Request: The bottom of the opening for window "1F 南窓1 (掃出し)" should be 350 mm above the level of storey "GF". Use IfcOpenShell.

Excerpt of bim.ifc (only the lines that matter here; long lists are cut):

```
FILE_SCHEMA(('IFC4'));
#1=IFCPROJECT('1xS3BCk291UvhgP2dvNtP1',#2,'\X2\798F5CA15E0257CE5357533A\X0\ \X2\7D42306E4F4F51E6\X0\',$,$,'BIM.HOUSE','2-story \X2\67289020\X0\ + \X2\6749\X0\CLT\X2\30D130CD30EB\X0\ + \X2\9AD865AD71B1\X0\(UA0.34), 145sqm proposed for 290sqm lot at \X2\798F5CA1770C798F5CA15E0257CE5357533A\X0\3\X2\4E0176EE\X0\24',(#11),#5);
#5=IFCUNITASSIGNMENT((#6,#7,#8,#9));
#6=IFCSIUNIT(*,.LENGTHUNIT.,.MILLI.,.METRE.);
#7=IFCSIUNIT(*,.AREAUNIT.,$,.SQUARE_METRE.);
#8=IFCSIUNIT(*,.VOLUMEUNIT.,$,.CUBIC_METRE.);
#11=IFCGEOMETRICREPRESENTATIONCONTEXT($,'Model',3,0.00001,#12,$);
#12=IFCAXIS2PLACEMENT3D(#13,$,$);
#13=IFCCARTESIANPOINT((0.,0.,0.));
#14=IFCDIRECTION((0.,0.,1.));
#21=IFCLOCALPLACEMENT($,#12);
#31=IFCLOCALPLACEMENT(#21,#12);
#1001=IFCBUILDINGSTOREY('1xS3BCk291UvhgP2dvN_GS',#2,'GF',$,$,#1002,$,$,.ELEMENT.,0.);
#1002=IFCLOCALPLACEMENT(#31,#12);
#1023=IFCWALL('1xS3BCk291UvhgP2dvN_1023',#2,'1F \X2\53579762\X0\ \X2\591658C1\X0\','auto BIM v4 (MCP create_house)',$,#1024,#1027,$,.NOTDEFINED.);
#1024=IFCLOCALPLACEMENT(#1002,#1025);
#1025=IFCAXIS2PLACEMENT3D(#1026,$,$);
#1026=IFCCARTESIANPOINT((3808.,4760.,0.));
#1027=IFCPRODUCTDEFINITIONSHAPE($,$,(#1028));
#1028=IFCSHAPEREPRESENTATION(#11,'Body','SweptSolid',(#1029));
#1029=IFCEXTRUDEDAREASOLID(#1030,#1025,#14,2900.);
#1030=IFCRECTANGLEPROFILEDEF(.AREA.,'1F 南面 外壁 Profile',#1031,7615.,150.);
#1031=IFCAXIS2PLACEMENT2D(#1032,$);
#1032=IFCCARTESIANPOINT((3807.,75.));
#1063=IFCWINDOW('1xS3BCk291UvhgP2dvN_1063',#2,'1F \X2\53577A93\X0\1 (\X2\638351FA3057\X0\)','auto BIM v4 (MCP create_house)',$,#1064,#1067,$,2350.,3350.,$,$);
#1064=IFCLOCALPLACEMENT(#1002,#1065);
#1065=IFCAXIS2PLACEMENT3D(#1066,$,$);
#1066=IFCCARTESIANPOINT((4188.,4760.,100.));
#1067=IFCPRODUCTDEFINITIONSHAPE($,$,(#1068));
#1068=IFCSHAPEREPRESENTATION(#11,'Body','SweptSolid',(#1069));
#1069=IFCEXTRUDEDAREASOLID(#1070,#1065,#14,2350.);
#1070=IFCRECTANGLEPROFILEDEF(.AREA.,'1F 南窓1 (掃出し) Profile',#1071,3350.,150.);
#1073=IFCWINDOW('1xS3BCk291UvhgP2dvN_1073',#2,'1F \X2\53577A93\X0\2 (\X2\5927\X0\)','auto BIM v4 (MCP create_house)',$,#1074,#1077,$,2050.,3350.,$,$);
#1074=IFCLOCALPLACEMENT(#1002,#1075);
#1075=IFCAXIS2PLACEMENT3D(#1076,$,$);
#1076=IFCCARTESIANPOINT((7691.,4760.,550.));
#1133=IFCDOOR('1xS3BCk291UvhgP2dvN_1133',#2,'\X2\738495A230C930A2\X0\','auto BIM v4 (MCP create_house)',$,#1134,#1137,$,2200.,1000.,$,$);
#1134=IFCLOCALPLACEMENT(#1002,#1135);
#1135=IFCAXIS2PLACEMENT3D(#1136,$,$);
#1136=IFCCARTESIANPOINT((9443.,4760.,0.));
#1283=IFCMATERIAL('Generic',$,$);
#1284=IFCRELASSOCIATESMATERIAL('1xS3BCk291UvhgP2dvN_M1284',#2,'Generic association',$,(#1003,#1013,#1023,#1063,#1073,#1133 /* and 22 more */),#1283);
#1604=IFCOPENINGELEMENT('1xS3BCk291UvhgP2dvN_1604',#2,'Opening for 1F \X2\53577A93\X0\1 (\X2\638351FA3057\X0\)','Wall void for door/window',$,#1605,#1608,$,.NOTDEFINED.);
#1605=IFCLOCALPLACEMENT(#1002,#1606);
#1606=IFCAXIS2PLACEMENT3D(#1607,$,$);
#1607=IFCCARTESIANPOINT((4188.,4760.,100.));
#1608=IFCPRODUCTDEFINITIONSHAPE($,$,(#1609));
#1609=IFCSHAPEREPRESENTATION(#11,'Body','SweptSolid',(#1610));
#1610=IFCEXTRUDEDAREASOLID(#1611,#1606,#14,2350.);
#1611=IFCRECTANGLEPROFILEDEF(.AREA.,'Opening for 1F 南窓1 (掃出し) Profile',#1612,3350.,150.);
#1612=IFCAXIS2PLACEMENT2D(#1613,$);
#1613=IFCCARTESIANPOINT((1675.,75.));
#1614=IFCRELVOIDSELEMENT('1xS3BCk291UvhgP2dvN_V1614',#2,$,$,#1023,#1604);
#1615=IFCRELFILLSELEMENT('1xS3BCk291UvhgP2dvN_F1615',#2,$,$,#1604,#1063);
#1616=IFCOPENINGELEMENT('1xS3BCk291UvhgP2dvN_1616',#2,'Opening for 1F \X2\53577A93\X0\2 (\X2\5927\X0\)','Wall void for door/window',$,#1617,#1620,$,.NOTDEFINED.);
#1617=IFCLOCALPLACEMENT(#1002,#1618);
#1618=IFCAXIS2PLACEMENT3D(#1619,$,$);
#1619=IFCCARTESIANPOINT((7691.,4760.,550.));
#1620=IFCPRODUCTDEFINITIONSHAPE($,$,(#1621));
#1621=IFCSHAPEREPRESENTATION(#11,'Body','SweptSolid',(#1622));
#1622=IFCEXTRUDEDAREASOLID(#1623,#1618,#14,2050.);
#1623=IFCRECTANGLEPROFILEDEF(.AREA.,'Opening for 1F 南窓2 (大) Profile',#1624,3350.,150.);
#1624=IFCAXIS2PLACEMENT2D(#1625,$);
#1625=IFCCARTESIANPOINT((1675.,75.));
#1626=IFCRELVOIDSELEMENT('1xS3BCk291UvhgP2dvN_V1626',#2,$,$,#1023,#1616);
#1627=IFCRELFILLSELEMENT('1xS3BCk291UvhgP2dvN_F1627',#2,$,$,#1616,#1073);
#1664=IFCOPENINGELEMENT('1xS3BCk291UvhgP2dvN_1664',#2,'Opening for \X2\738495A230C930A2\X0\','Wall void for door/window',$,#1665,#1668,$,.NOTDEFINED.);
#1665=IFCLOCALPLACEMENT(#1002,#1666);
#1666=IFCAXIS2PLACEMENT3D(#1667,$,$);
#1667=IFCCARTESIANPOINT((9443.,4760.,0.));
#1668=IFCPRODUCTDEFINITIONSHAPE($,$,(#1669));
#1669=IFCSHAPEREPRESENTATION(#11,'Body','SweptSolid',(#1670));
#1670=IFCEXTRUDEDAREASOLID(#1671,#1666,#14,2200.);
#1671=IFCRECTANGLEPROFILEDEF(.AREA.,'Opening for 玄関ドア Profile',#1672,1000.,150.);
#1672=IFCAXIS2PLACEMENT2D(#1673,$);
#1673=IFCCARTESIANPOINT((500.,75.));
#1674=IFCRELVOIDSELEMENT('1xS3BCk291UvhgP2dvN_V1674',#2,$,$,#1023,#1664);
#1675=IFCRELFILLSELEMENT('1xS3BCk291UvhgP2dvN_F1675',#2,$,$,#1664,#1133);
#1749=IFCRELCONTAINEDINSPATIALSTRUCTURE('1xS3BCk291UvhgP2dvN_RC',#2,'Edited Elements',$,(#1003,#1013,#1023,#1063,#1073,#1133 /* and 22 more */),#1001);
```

```python
import numpy as np
import ifcopenshell
import ifcopenshell.api.geometry
import ifcopenshell.geom
import ifcopenshell.util.element
import ifcopenshell.util.placement
import ifcopenshell.util.shape
import ifcopenshell.util.unit

model = ifcopenshell.open("bim.ifc")
unit_scale = ifcopenshell.util.unit.calculate_unit_scale(model)

window = model.by_id(1063)
opening = window.FillsVoids[0].RelatingOpeningElement
storey = ifcopenshell.util.element.get_container(window, ifc_class="IfcBuildingStorey")
level = ifcopenshell.util.placement.get_local_placement(storey.ObjectPlacement)[2, 3]

# The opening's origin need not be at the sill, so measure its lowest point.
shape = ifcopenshell.geom.create_shape(ifcopenshell.geom.settings(), opening)
bottom = ifcopenshell.util.shape.get_shape_bottom_elevation(shape, shape.geometry) / unit_scale
dz = level + 350.0 - bottom

shift = np.array([0.0, 0.0, dz])
# The window is not placed relative to its opening, so move both.
for product in (opening, window):
    matrix = ifcopenshell.util.placement.get_local_placement(product.ObjectPlacement)
    matrix[:3, 3] += shift
    ifcopenshell.api.geometry.edit_object_placement(model, product=product, matrix=matrix, is_si=False)

print(f"moved by {dz * unit_scale:+.3f} m")

model.write("bim_updated.ifc")
```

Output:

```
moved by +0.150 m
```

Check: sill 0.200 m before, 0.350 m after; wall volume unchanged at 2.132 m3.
